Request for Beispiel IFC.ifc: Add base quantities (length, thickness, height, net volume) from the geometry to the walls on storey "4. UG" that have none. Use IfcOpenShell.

First a look at what the model holds.

```python
import ifcopenshell
import ifcopenshell.util.element
import ifcopenshell.util.unit

model = ifcopenshell.open("Beispiel IFC.ifc")
print(model.schema)
for unit_type in ("LENGTHUNIT", "AREAUNIT", "VOLUMEUNIT"):
    print(unit_type, ifcopenshell.util.unit.calculate_unit_scale(model, unit_type))
storey = next(s for s in model.by_type("IfcBuildingStorey") if s.Name == "4. UG")
walls = [e for e in ifcopenshell.util.element.get_decomposition(storey) if e.is_a("IfcWall")]
for e in sorted(walls, key=lambda e: e.id()):
    print(e.id(), e.is_a(), e.Name, list(ifcopenshell.util.element.get_psets(e, qtos_only=True)), sep=" | ")
```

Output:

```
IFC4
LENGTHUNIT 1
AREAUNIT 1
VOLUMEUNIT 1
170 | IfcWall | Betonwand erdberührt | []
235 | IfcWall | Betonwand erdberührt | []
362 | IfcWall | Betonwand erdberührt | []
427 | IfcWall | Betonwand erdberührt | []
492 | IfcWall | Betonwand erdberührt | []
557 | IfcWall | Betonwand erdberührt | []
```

```python
import ifcopenshell
import ifcopenshell.api.pset
import ifcopenshell.geom
import ifcopenshell.util.element
import ifcopenshell.util.shape
import ifcopenshell.util.unit

model = ifcopenshell.open("Beispiel IFC.ifc")
unit_scale = ifcopenshell.util.unit.calculate_unit_scale(model)
volume_scale = ifcopenshell.util.unit.calculate_unit_scale(model, "VOLUMEUNIT")
settings = ifcopenshell.geom.settings()

storey = next(s for s in model.by_type("IfcBuildingStorey") if s.Name == "4. UG")
walls = [e for e in ifcopenshell.util.element.get_decomposition(storey) if e.is_a("IfcWall")]

for e in sorted(walls, key=lambda e: e.id()):
    if ifcopenshell.util.element.get_psets(e, qtos_only=True, should_inherit=False):
        continue
    # Geometry comes back in metres, in the element's own axes.
    shape = ifcopenshell.geom.create_shape(settings, e)
    values = {
        "Length": ifcopenshell.util.shape.get_x(shape.geometry) / unit_scale,
        "Width": ifcopenshell.util.shape.get_y(shape.geometry) / unit_scale,
        "Height": ifcopenshell.util.shape.get_z(shape.geometry) / unit_scale,
        "NetVolume": ifcopenshell.util.shape.get_volume(shape.geometry) / volume_scale,
    }
    qto = ifcopenshell.api.pset.add_qto(model, product=e, name="Qto_WallBaseQuantities")
    ifcopenshell.api.pset.edit_qto(model, qto=qto, properties=values)
    print(e.id(), {k: round(v, 3) for k, v in values.items()})

model.write("Beispiel IFC_updated.ifc")
```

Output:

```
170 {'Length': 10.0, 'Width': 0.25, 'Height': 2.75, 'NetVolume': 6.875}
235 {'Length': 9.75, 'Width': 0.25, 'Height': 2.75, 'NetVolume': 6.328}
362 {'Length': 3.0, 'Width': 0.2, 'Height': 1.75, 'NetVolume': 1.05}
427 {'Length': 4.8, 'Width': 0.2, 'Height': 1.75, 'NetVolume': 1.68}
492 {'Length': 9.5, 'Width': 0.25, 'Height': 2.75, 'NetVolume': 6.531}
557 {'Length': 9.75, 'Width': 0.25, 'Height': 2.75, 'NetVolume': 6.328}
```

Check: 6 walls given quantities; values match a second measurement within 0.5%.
